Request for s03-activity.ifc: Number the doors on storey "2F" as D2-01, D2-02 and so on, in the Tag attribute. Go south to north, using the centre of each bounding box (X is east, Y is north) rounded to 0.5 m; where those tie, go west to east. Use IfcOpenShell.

First a look at what the model holds.

```python
import ifcopenshell
import ifcopenshell.util.element
import ifcopenshell.util.placement

model = ifcopenshell.open("s03-activity.ifc")
print(model.schema)
storey = next(s for s in model.by_type("IfcBuildingStorey") if s.Name == "2F")
doors = [e for e in ifcopenshell.util.element.get_decomposition(storey) if e.is_a("IfcDoor")]
for e in sorted(doors, key=lambda e: e.id()):
    origin = ifcopenshell.util.placement.get_local_placement(e.ObjectPlacement)[:3, 3]
    print(e.id(), e.Tag, e.Name, origin.round(2) + 0.0, sep=" | ")
```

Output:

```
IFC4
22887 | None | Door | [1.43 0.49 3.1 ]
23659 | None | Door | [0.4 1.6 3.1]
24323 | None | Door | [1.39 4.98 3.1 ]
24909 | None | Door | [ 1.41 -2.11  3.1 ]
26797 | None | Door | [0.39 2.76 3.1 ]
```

```python
import ifcopenshell
import ifcopenshell.geom
import ifcopenshell.util.element
import ifcopenshell.util.shape

model = ifcopenshell.open("s03-activity.ifc")
settings = ifcopenshell.geom.settings()
settings.set("use-world-coords", True)


def centre(element):
    shape = ifcopenshell.geom.create_shape(settings, element)
    return ifcopenshell.util.shape.get_bbox_centroid(shape.geometry)


storey = next(s for s in model.by_type("IfcBuildingStorey") if s.Name == "2F")
doors = [e for e in ifcopenshell.util.element.get_decomposition(storey) if e.is_a("IfcDoor")]

# Insertion points can sit at a corner or the storey origin, so sort by the geometry (in metres).
centres = {e: centre(e) for e in doors}
doors.sort(key=lambda e: (round(centres[e][1] / 0.5), centres[e][0]))

for i, e in enumerate(doors, start=1):
    number = f"D2-{i:02d}"
    e.Tag = number
    print(e.id(), number)

model.write("s03-activity_v2.ifc")
```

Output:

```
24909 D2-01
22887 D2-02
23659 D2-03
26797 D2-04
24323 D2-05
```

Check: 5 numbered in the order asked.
